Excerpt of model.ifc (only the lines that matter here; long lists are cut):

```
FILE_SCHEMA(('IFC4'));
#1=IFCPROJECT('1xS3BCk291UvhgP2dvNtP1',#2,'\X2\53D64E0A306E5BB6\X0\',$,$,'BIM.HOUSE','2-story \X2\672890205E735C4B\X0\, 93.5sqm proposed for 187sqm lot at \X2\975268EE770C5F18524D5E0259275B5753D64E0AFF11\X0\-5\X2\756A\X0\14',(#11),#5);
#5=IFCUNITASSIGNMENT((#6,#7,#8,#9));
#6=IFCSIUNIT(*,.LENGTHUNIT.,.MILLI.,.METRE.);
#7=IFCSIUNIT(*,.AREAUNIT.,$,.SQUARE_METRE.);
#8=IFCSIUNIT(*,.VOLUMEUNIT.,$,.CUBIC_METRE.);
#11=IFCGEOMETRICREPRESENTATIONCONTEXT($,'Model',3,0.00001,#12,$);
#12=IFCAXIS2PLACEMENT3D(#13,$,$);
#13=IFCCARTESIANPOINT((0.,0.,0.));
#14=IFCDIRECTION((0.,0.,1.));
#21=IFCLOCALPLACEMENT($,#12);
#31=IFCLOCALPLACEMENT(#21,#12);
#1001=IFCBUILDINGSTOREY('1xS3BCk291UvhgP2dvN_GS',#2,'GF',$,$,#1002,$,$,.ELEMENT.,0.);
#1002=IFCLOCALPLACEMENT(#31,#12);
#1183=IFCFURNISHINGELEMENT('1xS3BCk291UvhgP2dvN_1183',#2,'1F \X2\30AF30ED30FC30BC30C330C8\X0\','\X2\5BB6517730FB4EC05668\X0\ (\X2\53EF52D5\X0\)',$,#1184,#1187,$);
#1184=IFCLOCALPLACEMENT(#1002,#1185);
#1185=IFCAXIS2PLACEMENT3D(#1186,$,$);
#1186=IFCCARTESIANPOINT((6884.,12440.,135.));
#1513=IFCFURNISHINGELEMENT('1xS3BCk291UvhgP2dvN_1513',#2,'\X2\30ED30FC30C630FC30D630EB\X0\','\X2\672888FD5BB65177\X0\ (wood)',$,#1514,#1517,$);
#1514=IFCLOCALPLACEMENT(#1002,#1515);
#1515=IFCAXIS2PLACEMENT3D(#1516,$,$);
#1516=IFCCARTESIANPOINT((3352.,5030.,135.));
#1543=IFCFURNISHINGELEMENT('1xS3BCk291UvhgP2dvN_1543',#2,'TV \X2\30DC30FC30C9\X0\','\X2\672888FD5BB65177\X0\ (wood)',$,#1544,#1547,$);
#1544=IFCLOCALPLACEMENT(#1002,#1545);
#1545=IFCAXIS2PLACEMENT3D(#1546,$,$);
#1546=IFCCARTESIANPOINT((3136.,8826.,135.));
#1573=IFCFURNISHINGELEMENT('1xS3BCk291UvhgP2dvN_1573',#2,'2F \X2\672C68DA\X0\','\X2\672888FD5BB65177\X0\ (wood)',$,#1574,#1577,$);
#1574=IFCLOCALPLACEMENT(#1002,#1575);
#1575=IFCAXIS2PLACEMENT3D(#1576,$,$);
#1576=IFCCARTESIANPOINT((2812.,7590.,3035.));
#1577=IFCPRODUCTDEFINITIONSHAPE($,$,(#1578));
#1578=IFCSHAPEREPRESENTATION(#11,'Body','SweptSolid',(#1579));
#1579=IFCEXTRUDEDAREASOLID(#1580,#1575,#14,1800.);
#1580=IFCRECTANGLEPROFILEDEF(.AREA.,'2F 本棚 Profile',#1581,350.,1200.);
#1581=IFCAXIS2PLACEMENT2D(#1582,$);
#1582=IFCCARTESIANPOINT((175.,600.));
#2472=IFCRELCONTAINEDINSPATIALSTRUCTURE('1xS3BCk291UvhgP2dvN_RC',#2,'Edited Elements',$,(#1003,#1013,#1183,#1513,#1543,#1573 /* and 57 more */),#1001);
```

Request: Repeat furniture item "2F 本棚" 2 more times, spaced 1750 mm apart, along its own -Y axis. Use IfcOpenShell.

```python
import ifcopenshell
import ifcopenshell.api.geometry
import ifcopenshell.api.root
import ifcopenshell.util.element
import ifcopenshell.util.placement
import ifcopenshell.util.unit

model = ifcopenshell.open("model.ifc")
unit_scale = ifcopenshell.util.unit.calculate_unit_scale(model)


def reuse_history(source, copy):
    """copy_class also copies each property set's owner history, people and application; keep the originals."""
    for rel in copy.IsDefinedBy:
        if rel.is_a("IfcRelDefinesByProperties") and (history := rel.RelatingPropertyDefinition.OwnerHistory):
            rel.RelatingPropertyDefinition.OwnerHistory = source.OwnerHistory
            ifcopenshell.util.element.remove_deep2(model, history)


source = model.by_guid("1xS3BCk291UvhgP2dvN_1573")
base = ifcopenshell.util.placement.get_local_placement(source.ObjectPlacement)
step = -base[:3, 1] * 1.75 / unit_scale

for i in range(1, 3):
    copy = ifcopenshell.api.root.copy_class(model, product=source)
    copy.Representation = ifcopenshell.util.element.copy_deep(
        model, source.Representation, exclude=["IfcGeometricRepresentationContext", "IfcRepresentationMap"]
    )
    reuse_history(source, copy)
    matrix = base.copy()
    matrix[:3, 3] += i * step
    print("added at", matrix[:3, 3].round(3) + 0.0)
    ifcopenshell.api.geometry.edit_object_placement(model, product=copy, matrix=matrix, is_si=False)

model.write("model_updated.ifc")
```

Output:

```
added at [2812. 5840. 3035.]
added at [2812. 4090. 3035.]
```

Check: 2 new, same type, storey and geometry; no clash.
